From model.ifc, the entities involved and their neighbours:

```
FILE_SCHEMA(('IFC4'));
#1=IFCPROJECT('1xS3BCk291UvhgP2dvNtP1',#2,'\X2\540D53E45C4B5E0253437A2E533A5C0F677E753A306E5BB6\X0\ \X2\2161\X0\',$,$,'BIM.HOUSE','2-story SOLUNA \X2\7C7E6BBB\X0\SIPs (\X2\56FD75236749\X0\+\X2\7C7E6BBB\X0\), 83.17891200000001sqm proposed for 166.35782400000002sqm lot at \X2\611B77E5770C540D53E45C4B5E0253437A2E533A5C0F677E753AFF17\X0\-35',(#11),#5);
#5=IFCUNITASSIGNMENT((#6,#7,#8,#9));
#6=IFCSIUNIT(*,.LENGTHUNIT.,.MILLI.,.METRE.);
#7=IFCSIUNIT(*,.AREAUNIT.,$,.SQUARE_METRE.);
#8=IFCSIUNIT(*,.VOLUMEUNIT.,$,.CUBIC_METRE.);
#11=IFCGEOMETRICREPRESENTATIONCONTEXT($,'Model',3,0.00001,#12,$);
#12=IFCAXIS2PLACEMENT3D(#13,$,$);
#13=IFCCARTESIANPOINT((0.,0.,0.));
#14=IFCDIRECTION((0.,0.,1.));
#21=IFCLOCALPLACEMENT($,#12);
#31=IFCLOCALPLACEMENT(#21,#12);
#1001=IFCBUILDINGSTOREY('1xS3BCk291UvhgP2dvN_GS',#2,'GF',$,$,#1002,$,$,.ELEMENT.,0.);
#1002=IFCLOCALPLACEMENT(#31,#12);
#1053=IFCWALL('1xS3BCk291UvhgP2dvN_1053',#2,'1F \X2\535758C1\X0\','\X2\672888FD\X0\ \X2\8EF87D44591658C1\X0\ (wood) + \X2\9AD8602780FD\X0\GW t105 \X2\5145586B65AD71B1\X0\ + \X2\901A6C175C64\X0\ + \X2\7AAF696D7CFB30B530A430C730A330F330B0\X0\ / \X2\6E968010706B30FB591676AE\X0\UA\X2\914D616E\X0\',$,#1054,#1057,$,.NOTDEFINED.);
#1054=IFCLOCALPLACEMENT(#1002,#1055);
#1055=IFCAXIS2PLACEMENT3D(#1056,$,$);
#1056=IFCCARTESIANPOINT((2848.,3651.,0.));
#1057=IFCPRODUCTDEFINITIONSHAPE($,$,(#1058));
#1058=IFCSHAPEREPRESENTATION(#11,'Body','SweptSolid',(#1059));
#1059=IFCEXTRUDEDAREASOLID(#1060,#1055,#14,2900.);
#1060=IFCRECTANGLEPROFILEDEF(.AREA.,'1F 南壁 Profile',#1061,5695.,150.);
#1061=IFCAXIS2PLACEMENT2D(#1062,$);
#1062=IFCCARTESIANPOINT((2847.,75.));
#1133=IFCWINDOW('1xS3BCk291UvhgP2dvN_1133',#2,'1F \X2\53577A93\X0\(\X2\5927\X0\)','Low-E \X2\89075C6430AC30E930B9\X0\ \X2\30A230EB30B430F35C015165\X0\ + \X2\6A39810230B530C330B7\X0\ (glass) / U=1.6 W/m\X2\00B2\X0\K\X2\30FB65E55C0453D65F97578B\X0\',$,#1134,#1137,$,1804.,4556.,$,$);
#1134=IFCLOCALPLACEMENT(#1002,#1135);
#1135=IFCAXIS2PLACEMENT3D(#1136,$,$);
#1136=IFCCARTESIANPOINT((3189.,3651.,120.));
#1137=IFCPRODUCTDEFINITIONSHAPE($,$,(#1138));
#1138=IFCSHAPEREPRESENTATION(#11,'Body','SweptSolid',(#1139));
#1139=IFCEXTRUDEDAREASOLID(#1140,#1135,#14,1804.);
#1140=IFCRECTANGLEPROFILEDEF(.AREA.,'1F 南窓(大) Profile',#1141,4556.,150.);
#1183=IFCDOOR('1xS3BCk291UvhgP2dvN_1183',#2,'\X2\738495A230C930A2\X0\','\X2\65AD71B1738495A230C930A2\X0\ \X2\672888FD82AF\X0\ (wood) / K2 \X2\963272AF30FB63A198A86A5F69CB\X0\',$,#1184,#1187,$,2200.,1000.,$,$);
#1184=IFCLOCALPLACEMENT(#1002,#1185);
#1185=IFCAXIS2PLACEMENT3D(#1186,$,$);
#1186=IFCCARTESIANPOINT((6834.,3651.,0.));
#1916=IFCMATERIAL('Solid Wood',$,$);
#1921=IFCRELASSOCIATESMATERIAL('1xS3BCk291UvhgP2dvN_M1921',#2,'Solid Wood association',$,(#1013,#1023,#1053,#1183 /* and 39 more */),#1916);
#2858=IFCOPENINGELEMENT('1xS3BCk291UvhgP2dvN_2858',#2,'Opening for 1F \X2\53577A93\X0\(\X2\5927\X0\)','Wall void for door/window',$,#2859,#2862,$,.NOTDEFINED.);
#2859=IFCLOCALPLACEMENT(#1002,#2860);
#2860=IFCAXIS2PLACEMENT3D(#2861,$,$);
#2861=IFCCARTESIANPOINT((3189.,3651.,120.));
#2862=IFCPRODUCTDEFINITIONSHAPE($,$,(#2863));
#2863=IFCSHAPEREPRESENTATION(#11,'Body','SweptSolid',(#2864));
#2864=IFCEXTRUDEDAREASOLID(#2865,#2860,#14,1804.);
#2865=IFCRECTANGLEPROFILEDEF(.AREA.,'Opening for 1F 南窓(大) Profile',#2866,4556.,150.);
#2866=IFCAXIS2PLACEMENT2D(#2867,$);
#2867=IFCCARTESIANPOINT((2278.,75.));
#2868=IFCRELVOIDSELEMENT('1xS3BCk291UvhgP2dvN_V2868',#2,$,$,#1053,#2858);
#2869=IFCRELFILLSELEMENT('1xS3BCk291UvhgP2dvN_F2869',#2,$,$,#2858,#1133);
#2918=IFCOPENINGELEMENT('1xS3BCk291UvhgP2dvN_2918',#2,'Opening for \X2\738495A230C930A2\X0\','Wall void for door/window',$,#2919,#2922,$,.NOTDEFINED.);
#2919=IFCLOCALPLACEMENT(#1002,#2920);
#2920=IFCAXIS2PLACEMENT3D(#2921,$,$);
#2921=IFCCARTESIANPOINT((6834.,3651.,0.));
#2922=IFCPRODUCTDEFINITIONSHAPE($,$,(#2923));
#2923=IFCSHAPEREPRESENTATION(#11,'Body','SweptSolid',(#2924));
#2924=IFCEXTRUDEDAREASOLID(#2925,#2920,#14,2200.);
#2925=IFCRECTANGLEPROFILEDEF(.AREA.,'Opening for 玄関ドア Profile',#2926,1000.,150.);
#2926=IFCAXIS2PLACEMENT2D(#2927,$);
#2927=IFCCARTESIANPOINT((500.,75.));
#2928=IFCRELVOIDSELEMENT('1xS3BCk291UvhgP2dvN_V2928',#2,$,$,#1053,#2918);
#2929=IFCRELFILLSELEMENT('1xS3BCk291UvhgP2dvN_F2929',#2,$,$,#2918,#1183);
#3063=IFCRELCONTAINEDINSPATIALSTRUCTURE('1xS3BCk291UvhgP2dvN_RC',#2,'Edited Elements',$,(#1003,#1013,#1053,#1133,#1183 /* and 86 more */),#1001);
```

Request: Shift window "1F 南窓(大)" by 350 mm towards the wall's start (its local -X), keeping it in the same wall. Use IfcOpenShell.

```python
import ifcopenshell
import ifcopenshell.api.geometry
import ifcopenshell.util.placement
import ifcopenshell.util.unit

model = ifcopenshell.open("model.ifc")
unit_scale = ifcopenshell.util.unit.calculate_unit_scale(model)

window = model.by_id(1133)
opening = window.FillsVoids[0].RelatingOpeningElement
wall = opening.VoidsElements[0].RelatingBuildingElement

wall_matrix = ifcopenshell.util.placement.get_local_placement(wall.ObjectPlacement)
shift = wall_matrix[:3, 0] * -0.35 / unit_scale
before = ifcopenshell.util.placement.get_local_placement(window.ObjectPlacement)[:3, 3].copy()

# The window is not placed relative to its opening, so move both.
for product in (opening, window):
    matrix = ifcopenshell.util.placement.get_local_placement(product.ObjectPlacement)
    matrix[:3, 3] += shift
    ifcopenshell.api.geometry.edit_object_placement(model, product=product, matrix=matrix, is_si=False)

after = ifcopenshell.util.placement.get_local_placement(window.ObjectPlacement)[:3, 3]
print("window moved by", (after - before).round(3) + 0.0)

model.write("model_updated.ifc")
```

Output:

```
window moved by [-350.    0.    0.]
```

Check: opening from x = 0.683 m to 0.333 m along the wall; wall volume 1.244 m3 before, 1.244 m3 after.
